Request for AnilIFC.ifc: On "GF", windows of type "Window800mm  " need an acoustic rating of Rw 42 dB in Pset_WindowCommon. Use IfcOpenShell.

First a look at what the model holds.

```python
import ifcopenshell
import ifcopenshell.util.element

model = ifcopenshell.open("AnilIFC.ifc")
print(model.schema)
storey = next(s for s in model.by_type("IfcBuildingStorey") if s.Name == "GF")
windows = [e for e in ifcopenshell.util.element.get_decomposition(storey) if e.is_a("IfcWindow")]
seen = {}
for e in windows:
    element_type = ifcopenshell.util.element.get_type(e)
    key = (element_type.Name if element_type != e and element_type else None, ifcopenshell.util.element.get_pset(e, "Pset_WindowCommon", "AcousticRating"))
    seen[key] = seen.get(key, 0) + 1
for (name, value), count in sorted(seen.items(), key=str):
    print(count, "x", name, "|", value)
```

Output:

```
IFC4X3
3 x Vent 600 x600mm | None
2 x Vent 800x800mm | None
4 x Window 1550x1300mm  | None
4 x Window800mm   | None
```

```python
import ifcopenshell
import ifcopenshell.api.pset
import ifcopenshell.util.element

model = ifcopenshell.open("AnilIFC.ifc")

storey = next(s for s in model.by_type("IfcBuildingStorey") if s.Name == "GF")
windows = [e for e in ifcopenshell.util.element.get_decomposition(storey) if e.is_a("IfcWindow")]

count = 0
for e in windows:
    element_type = ifcopenshell.util.element.get_type(e)
    if element_type in (None, e) or element_type.Name != "Window800mm  ":
        continue
    # add_pset returns the element's existing set when there is one.
    pset = ifcopenshell.api.pset.add_pset(model, product=e, name="Pset_WindowCommon")
    ifcopenshell.api.pset.edit_pset(model, pset=pset, properties={"AcousticRating": "Rw 42 dB"})
    count += 1

print(count, "windows updated")

model.write("AnilIFC_rev.ifc")
```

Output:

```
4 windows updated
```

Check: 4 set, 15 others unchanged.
